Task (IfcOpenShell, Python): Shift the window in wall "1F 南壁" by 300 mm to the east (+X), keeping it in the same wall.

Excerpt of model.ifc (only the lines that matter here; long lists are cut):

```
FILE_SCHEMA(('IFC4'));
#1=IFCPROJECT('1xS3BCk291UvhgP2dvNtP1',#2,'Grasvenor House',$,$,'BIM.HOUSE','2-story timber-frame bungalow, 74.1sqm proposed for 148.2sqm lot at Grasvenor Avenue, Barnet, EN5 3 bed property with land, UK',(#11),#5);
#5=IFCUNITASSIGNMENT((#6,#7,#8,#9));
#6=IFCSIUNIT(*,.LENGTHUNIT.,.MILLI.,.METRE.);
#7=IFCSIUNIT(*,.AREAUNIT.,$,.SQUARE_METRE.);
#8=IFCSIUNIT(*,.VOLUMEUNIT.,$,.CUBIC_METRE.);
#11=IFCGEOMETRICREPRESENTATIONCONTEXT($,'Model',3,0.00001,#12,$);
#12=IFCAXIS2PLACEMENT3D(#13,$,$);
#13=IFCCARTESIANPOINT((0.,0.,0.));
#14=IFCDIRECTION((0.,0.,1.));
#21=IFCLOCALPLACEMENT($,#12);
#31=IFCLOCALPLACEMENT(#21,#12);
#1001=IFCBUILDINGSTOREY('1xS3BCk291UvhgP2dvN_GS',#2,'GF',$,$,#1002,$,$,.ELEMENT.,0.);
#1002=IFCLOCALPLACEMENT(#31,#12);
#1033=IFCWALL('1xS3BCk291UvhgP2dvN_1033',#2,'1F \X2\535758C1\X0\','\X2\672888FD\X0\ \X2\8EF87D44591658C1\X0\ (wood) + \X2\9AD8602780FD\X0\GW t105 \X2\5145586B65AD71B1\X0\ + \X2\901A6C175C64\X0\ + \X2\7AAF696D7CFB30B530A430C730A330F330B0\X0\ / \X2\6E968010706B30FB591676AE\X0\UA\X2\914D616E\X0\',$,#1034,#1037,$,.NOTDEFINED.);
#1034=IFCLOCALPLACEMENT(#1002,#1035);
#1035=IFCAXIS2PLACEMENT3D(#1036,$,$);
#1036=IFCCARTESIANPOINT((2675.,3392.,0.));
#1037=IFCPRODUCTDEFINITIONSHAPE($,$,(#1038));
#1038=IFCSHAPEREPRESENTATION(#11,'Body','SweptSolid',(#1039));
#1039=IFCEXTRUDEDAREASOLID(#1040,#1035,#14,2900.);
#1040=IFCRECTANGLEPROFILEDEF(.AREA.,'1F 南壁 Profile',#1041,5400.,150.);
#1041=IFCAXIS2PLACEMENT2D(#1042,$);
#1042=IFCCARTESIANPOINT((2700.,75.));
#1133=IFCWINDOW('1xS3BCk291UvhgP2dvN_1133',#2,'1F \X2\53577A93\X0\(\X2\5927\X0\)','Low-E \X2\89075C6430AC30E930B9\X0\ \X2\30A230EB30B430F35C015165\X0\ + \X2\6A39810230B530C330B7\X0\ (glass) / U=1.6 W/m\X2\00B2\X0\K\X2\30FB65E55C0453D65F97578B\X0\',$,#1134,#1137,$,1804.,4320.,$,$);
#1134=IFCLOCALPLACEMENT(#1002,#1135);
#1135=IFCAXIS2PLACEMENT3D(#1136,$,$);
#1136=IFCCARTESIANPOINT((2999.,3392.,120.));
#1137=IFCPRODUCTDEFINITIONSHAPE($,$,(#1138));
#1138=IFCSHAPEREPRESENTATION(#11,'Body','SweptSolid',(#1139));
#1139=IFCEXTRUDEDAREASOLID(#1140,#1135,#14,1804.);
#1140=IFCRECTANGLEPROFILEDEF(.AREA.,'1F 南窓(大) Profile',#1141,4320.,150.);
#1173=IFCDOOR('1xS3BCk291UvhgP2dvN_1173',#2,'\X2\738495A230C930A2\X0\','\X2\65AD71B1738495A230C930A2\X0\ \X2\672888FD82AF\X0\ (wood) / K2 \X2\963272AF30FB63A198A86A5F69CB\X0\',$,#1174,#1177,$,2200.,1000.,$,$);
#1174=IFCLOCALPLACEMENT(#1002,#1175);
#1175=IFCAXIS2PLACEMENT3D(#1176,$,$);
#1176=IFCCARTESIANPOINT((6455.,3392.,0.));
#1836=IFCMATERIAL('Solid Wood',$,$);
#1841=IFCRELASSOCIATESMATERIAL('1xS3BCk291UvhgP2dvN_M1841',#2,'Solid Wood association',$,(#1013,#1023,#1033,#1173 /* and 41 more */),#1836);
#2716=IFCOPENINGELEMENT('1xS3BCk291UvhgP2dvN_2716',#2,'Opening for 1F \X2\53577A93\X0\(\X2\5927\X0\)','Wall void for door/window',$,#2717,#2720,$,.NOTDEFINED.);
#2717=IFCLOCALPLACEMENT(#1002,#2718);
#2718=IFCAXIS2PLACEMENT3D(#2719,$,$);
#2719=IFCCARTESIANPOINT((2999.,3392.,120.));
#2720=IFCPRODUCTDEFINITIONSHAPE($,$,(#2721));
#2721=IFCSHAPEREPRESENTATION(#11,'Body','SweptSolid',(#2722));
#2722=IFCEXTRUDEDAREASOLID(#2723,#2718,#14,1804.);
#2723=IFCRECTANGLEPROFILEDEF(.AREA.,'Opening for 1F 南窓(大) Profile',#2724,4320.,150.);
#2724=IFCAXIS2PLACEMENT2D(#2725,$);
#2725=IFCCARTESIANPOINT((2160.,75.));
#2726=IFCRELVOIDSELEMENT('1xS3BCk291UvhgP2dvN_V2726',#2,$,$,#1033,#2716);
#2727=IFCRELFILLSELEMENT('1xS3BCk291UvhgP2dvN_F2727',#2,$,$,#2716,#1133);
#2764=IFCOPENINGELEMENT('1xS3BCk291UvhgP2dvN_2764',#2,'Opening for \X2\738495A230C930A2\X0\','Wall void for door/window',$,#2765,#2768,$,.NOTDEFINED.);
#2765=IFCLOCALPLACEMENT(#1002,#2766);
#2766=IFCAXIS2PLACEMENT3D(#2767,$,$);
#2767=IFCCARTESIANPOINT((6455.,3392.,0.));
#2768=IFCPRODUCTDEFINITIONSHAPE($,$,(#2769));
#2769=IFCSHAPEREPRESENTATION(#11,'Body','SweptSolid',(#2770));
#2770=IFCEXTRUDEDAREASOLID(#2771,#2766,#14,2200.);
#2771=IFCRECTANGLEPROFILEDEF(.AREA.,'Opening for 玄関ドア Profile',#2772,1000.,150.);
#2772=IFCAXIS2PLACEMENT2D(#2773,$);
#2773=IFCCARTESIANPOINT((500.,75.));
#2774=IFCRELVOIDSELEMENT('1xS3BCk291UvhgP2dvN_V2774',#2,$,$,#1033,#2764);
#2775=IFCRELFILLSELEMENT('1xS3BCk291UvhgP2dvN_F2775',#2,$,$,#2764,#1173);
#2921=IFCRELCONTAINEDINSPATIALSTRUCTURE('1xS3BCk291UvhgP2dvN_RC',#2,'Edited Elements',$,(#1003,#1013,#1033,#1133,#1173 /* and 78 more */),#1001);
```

```python
import ifcopenshell
import ifcopenshell.api.geometry
import ifcopenshell.util.placement

model = ifcopenshell.open("model.ifc")

window = model.by_guid("1xS3BCk291UvhgP2dvN_1133")
opening = window.FillsVoids[0].RelatingOpeningElement
wall = opening.VoidsElements[0].RelatingBuildingElement

wall_matrix = ifcopenshell.util.placement.get_local_placement(wall.ObjectPlacement)
shift = wall_matrix[:3, 0] * 300.0
before = ifcopenshell.util.placement.get_local_placement(window.ObjectPlacement)[:3, 3].copy()

# The window is not placed relative to its opening, so move both.
for product in (opening, window):
    matrix = ifcopenshell.util.placement.get_local_placement(product.ObjectPlacement)
    matrix[:3, 3] += shift
    ifcopenshell.api.geometry.edit_object_placement(model, product=product, matrix=matrix, is_si=False)

after = ifcopenshell.util.placement.get_local_placement(window.ObjectPlacement)[:3, 3]
print("window moved by", (after - before).round(3) + 0.0)

model.write("model_v2.ifc")
```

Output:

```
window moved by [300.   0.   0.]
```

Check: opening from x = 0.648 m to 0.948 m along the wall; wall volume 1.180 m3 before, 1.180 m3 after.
